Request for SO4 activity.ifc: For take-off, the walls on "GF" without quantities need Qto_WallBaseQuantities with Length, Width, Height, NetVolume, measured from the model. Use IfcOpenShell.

First a look at what the model holds.

```python
import ifcopenshell
import ifcopenshell.util.element
import ifcopenshell.util.unit

model = ifcopenshell.open("SO4 activity.ifc")
print(model.schema)
for unit_type in ("LENGTHUNIT", "AREAUNIT", "VOLUMEUNIT"):
    print(unit_type, ifcopenshell.util.unit.calculate_unit_scale(model, unit_type))
storey = next(s for s in model.by_type("IfcBuildingStorey") if s.Name == "GF")
walls = [e for e in ifcopenshell.util.element.get_decomposition(storey) if e.is_a("IfcWall")]
for e in sorted(walls, key=lambda e: e.id()):
    print(e.id(), e.is_a(), e.Name, list(ifcopenshell.util.element.get_psets(e, qtos_only=True)), sep=" | ")
```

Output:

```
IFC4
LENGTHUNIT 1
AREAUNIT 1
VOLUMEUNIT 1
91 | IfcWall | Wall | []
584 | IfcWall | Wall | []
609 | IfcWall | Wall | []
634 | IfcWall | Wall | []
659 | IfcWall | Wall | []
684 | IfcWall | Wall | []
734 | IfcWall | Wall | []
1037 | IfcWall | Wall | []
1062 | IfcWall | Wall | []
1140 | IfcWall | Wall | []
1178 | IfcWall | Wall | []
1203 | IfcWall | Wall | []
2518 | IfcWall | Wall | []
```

```python
import ifcopenshell
import ifcopenshell.api.pset
import ifcopenshell.geom
import ifcopenshell.util.element
import ifcopenshell.util.shape
import ifcopenshell.util.unit

model = ifcopenshell.open("SO4 activity.ifc")
unit_scale = ifcopenshell.util.unit.calculate_unit_scale(model)
volume_scale = ifcopenshell.util.unit.calculate_unit_scale(model, "VOLUMEUNIT")
settings = ifcopenshell.geom.settings()

storey = next(s for s in model.by_type("IfcBuildingStorey") if s.Name == "GF")
walls = [e for e in ifcopenshell.util.element.get_decomposition(storey) if e.is_a("IfcWall")]

for e in sorted(walls, key=lambda e: e.id()):
    if ifcopenshell.util.element.get_psets(e, qtos_only=True, should_inherit=False):
        continue
    # Geometry comes back in metres, in the element's own axes.
    shape = ifcopenshell.geom.create_shape(settings, e)
    values = {
        "Length": ifcopenshell.util.shape.get_x(shape.geometry) / unit_scale,
        "Width": ifcopenshell.util.shape.get_y(shape.geometry) / unit_scale,
        "Height": ifcopenshell.util.shape.get_z(shape.geometry) / unit_scale,
        "NetVolume": ifcopenshell.util.shape.get_volume(shape.geometry) / volume_scale,
    }
    qto = ifcopenshell.api.pset.add_qto(model, product=e, name="Qto_WallBaseQuantities")
    ifcopenshell.api.pset.edit_qto(model, qto=qto, properties=values)
    print(e.id(), {k: round(v, 3) for k, v in values.items()})

model.write("SO4 activity_v2.ifc")
```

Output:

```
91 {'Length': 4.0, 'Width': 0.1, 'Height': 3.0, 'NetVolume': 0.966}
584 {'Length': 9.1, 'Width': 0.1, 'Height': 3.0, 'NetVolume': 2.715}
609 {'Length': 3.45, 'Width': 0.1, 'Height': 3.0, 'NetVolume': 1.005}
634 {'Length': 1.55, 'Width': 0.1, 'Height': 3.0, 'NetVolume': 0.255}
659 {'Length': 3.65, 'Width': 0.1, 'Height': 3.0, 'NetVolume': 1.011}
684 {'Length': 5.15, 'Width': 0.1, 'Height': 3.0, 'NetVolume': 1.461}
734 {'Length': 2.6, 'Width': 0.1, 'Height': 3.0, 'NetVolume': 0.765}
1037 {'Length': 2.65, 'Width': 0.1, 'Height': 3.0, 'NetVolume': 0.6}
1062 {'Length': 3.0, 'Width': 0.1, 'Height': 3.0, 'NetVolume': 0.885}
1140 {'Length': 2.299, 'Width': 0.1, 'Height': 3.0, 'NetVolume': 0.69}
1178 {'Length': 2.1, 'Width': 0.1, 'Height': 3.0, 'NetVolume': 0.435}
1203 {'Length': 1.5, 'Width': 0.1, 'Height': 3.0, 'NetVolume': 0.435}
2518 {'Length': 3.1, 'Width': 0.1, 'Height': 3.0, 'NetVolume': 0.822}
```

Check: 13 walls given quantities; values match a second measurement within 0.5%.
